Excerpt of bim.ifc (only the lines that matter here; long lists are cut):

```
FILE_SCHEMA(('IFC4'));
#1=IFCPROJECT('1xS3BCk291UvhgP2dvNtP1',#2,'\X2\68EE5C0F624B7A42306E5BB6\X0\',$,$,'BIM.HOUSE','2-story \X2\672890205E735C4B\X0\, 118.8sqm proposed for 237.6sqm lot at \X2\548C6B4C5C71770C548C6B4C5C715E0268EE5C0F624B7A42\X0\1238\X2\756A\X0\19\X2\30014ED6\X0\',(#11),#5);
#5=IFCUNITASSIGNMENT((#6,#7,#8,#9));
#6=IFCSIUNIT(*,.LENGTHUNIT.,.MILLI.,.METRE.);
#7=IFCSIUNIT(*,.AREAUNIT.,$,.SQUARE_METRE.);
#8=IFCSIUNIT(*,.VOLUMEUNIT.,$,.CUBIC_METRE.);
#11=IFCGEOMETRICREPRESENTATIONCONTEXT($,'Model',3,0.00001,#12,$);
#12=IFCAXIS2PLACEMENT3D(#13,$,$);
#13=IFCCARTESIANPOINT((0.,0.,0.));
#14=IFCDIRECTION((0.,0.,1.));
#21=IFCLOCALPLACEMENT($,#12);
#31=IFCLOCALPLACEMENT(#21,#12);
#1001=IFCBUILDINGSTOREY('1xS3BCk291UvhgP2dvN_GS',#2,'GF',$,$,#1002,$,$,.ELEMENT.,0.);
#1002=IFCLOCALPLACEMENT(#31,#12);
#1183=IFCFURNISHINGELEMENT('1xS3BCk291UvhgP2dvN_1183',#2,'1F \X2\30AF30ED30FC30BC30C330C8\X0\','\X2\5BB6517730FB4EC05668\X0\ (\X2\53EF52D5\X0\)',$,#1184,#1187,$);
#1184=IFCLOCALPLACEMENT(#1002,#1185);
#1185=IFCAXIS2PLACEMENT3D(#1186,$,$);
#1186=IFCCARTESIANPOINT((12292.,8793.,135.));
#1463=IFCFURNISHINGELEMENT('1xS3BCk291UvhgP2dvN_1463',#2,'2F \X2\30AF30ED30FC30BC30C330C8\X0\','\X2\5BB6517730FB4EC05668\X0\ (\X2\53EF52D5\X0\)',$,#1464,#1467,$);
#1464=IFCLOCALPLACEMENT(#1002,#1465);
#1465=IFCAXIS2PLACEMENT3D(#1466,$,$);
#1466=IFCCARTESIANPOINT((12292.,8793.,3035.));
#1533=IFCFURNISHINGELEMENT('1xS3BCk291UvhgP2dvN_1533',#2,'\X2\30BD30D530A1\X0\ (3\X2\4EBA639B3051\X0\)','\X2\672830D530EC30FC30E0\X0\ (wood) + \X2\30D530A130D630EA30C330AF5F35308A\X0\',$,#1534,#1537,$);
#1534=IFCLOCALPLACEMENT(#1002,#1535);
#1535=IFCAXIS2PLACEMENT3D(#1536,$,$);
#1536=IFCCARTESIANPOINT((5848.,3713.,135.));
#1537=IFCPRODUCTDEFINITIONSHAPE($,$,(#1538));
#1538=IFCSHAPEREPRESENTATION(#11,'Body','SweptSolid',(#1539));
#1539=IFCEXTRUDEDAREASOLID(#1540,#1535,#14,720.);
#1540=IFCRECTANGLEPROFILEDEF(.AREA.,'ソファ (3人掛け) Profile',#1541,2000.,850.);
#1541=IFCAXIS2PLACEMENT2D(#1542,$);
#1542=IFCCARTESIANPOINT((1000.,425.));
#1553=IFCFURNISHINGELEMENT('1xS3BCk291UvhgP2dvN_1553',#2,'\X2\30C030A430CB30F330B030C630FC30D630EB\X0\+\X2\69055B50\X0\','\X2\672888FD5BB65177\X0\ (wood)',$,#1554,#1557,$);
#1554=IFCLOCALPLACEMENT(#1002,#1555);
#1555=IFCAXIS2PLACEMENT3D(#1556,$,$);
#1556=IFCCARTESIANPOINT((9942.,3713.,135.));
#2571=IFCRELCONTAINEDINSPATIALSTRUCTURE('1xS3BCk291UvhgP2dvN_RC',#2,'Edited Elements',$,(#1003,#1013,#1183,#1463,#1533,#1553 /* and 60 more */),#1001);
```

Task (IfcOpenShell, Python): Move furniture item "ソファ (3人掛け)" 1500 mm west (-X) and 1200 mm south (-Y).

```python
import ifcopenshell
import ifcopenshell.api.geometry
import ifcopenshell.util.placement

model = ifcopenshell.open("bim.ifc")

item = model.by_id(1533)
matrix = ifcopenshell.util.placement.get_local_placement(item.ObjectPlacement)
matrix[0, 3] -= 1500.0
matrix[1, 3] -= 1200.0
ifcopenshell.api.geometry.edit_object_placement(model, product=item, matrix=matrix, is_si=False)

print(ifcopenshell.util.placement.get_local_placement(item.ObjectPlacement).round(3) + 0.0)

model.write("bim_updated.ifc")
```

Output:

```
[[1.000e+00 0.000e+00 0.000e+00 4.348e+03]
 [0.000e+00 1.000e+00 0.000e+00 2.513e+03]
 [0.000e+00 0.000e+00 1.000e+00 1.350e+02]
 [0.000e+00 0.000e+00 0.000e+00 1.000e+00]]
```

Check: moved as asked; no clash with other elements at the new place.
